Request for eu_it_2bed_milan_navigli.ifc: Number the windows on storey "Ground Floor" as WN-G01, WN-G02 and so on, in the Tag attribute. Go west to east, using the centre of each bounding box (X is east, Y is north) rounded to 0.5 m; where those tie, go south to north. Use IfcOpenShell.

First a look at what the model holds.

```python
import ifcopenshell
import ifcopenshell.util.element
import ifcopenshell.util.placement

model = ifcopenshell.open("eu_it_2bed_milan_navigli.ifc")
print(model.schema)
storey = next(s for s in model.by_type("IfcBuildingStorey") if s.Name == "Ground Floor")
windows = [e for e in ifcopenshell.util.element.get_decomposition(storey) if e.is_a("IfcWindow")]
for e in sorted(windows, key=lambda e: e.id()):
    origin = ifcopenshell.util.placement.get_local_placement(e.ObjectPlacement)[:3, 3]
    print(e.id(), e.Tag, e.Name, origin.round(2) + 0.0, sep=" | ")
```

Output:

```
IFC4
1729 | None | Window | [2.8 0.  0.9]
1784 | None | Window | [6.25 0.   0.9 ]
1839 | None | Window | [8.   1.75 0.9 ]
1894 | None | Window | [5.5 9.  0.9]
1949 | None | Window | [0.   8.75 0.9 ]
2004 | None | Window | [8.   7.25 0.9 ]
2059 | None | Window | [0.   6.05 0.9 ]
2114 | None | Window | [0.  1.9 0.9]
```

```python
import ifcopenshell
import ifcopenshell.geom
import ifcopenshell.util.element
import ifcopenshell.util.shape

model = ifcopenshell.open("eu_it_2bed_milan_navigli.ifc")
settings = ifcopenshell.geom.settings()
settings.set("use-world-coords", True)


def centre(element):
    shape = ifcopenshell.geom.create_shape(settings, element)
    return ifcopenshell.util.shape.get_bbox_centroid(shape.geometry)


storey = next(s for s in model.by_type("IfcBuildingStorey") if s.Name == "Ground Floor")
windows = [e for e in ifcopenshell.util.element.get_decomposition(storey) if e.is_a("IfcWindow")]

# Insertion points can sit at a corner or the storey origin, so sort by the geometry (in metres).
centres = {e: centre(e) for e in windows}
windows.sort(key=lambda e: (round(centres[e][0] / 0.5), centres[e][1]))

for i, e in enumerate(windows, start=1):
    number = f"WN-G{i:02d}"
    e.Tag = number
    print(e.id(), number)

model.write("eu_it_2bed_milan_navigli-out.ifc")
```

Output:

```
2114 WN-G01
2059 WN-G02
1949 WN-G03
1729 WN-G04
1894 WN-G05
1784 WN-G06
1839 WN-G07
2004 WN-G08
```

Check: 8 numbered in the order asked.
